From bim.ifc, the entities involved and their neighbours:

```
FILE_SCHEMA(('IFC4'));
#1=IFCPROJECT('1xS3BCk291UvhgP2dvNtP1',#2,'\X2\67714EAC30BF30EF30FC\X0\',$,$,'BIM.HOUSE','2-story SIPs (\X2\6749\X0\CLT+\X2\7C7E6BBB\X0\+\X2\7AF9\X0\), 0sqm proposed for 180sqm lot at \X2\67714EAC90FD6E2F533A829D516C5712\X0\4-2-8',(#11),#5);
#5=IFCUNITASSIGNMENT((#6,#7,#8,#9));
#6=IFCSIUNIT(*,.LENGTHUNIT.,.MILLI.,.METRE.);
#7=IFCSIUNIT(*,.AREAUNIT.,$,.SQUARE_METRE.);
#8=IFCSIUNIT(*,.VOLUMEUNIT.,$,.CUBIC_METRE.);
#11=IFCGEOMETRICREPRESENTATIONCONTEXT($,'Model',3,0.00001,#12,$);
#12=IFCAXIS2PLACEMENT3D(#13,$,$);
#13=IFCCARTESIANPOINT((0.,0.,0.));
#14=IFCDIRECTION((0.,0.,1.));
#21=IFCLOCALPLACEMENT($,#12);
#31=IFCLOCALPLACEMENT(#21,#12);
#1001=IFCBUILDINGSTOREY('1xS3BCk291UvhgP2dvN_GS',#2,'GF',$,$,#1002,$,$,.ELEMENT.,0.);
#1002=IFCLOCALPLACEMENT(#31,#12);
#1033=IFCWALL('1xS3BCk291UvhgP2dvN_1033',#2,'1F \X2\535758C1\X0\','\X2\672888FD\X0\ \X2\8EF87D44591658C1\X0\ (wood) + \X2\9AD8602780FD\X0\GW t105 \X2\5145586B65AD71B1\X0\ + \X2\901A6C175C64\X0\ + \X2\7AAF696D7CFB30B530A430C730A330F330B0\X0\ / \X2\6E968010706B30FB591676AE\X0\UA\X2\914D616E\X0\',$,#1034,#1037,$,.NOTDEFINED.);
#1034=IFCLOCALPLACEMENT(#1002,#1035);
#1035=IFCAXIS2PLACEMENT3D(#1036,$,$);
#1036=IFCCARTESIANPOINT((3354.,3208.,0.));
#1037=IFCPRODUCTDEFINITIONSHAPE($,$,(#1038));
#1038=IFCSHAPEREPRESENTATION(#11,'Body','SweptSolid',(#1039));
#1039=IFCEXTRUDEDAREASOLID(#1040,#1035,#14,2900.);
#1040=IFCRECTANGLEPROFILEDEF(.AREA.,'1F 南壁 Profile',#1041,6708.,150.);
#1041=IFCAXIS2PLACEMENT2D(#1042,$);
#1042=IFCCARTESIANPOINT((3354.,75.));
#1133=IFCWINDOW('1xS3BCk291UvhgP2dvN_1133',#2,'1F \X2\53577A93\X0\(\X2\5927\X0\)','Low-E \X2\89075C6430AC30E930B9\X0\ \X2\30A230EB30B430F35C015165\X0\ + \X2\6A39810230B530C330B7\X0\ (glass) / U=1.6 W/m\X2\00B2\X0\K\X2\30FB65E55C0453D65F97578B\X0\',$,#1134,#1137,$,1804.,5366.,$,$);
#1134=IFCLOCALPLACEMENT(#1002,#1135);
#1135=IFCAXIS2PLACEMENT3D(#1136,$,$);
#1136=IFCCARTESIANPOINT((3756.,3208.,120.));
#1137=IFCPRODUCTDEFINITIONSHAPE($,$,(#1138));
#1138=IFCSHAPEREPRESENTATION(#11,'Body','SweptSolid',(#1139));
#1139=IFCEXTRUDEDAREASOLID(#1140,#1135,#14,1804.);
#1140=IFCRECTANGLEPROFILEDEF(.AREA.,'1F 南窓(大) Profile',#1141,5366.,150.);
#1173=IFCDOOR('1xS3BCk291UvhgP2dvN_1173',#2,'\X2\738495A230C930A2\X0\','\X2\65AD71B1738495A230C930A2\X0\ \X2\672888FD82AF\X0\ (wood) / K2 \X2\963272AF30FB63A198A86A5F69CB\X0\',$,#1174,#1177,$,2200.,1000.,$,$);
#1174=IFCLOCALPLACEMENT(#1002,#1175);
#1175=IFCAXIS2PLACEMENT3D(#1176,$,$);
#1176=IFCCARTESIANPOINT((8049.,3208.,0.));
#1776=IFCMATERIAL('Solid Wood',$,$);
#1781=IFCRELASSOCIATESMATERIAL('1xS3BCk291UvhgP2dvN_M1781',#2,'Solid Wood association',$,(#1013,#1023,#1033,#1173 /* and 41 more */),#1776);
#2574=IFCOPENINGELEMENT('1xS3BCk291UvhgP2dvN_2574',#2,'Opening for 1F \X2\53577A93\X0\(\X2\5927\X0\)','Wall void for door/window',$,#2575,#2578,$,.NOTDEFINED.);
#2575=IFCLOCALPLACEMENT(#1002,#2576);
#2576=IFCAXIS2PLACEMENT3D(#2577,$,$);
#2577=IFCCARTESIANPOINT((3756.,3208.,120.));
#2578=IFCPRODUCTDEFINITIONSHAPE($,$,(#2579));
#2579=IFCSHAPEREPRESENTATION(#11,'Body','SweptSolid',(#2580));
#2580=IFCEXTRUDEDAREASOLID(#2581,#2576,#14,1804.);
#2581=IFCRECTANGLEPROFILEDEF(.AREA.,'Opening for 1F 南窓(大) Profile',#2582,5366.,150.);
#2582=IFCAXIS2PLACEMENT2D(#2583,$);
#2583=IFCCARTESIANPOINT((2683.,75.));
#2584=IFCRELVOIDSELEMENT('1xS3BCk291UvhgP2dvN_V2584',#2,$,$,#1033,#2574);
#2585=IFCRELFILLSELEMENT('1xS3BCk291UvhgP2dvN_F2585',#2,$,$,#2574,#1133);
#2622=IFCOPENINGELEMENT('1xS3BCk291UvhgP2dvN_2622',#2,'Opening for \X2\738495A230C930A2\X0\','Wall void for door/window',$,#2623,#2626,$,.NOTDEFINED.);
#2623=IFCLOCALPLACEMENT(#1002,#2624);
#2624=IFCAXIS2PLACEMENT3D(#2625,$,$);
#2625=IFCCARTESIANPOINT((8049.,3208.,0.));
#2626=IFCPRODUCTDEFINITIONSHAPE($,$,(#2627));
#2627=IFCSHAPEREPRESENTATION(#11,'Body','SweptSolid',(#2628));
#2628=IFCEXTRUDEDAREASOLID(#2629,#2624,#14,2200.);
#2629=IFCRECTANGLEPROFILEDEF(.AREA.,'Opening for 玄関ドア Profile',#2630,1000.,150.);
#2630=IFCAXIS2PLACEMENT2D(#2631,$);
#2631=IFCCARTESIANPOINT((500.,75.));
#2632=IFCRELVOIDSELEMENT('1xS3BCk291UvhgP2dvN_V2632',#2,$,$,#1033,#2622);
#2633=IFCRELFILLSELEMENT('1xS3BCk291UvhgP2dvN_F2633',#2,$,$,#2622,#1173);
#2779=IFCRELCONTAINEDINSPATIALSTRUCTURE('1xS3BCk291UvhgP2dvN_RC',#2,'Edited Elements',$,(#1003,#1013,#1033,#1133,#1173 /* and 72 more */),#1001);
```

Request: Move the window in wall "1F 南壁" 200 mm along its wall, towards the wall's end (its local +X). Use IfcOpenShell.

```python
import ifcopenshell
import ifcopenshell.api.geometry
import ifcopenshell.util.placement
import ifcopenshell.util.unit

model = ifcopenshell.open("bim.ifc")
unit_scale = ifcopenshell.util.unit.calculate_unit_scale(model)

window = model.by_guid("1xS3BCk291UvhgP2dvN_1133")
opening = window.FillsVoids[0].RelatingOpeningElement
wall = opening.VoidsElements[0].RelatingBuildingElement

wall_matrix = ifcopenshell.util.placement.get_local_placement(wall.ObjectPlacement)
shift = wall_matrix[:3, 0] * 0.2 / unit_scale
before = ifcopenshell.util.placement.get_local_placement(window.ObjectPlacement)[:3, 3].copy()

# The window is not placed relative to its opening, so move both.
for product in (opening, window):
    matrix = ifcopenshell.util.placement.get_local_placement(product.ObjectPlacement)
    matrix[:3, 3] += shift
    ifcopenshell.api.geometry.edit_object_placement(model, product=product, matrix=matrix, is_si=False)

after = ifcopenshell.util.placement.get_local_placement(window.ObjectPlacement)[:3, 3]
print("window moved by", (after - before).round(3) + 0.0)

model.write("bim_rev.ifc")
```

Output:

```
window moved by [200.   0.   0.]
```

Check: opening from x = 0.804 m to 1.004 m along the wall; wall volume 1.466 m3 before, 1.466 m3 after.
